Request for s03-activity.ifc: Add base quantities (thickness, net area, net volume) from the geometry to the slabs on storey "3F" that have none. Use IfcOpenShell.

First a look at what the model holds.

```python
import ifcopenshell
import ifcopenshell.util.element
import ifcopenshell.util.unit

model = ifcopenshell.open("s03-activity.ifc")
print(model.schema)
for unit_type in ("LENGTHUNIT", "AREAUNIT", "VOLUMEUNIT"):
    print(unit_type, ifcopenshell.util.unit.calculate_unit_scale(model, unit_type))
storey = next(s for s in model.by_type("IfcBuildingStorey") if s.Name == "3F")
slabs = [e for e in ifcopenshell.util.element.get_decomposition(storey) if e.is_a("IfcSlab")]
for e in sorted(slabs, key=lambda e: e.id()):
    print(e.id(), e.is_a(), e.Name, list(ifcopenshell.util.element.get_psets(e, qtos_only=True)), sep=" | ")
```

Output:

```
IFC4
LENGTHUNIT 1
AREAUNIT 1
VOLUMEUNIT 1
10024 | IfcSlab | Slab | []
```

```python
import ifcopenshell
import ifcopenshell.api.pset
import ifcopenshell.geom
import ifcopenshell.util.element
import ifcopenshell.util.shape
import ifcopenshell.util.unit

model = ifcopenshell.open("s03-activity.ifc")
unit_scale = ifcopenshell.util.unit.calculate_unit_scale(model)
area_scale = ifcopenshell.util.unit.calculate_unit_scale(model, "AREAUNIT")
volume_scale = ifcopenshell.util.unit.calculate_unit_scale(model, "VOLUMEUNIT")
settings = ifcopenshell.geom.settings()

storey = next(s for s in model.by_type("IfcBuildingStorey") if s.Name == "3F")
slabs = [e for e in ifcopenshell.util.element.get_decomposition(storey) if e.is_a("IfcSlab")]

for e in sorted(slabs, key=lambda e: e.id()):
    if ifcopenshell.util.element.get_psets(e, qtos_only=True, should_inherit=False):
        continue
    # Geometry comes back in metres, in the element's own axes.
    shape = ifcopenshell.geom.create_shape(settings, e)
    values = {
        "Width": ifcopenshell.util.shape.get_z(shape.geometry) / unit_scale,
        "NetArea": ifcopenshell.util.shape.get_footprint_area(shape.geometry) / area_scale,
        "NetVolume": ifcopenshell.util.shape.get_volume(shape.geometry) / volume_scale,
    }
    qto = ifcopenshell.api.pset.add_qto(model, product=e, name="Qto_SlabBaseQuantities")
    ifcopenshell.api.pset.edit_qto(model, qto=qto, properties=values)
    print(e.id(), {k: round(v, 3) for k, v in values.items()})

model.write("s03-activity-out.ifc")
```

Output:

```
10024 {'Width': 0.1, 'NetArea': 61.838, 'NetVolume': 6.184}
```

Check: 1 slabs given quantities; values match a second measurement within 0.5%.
